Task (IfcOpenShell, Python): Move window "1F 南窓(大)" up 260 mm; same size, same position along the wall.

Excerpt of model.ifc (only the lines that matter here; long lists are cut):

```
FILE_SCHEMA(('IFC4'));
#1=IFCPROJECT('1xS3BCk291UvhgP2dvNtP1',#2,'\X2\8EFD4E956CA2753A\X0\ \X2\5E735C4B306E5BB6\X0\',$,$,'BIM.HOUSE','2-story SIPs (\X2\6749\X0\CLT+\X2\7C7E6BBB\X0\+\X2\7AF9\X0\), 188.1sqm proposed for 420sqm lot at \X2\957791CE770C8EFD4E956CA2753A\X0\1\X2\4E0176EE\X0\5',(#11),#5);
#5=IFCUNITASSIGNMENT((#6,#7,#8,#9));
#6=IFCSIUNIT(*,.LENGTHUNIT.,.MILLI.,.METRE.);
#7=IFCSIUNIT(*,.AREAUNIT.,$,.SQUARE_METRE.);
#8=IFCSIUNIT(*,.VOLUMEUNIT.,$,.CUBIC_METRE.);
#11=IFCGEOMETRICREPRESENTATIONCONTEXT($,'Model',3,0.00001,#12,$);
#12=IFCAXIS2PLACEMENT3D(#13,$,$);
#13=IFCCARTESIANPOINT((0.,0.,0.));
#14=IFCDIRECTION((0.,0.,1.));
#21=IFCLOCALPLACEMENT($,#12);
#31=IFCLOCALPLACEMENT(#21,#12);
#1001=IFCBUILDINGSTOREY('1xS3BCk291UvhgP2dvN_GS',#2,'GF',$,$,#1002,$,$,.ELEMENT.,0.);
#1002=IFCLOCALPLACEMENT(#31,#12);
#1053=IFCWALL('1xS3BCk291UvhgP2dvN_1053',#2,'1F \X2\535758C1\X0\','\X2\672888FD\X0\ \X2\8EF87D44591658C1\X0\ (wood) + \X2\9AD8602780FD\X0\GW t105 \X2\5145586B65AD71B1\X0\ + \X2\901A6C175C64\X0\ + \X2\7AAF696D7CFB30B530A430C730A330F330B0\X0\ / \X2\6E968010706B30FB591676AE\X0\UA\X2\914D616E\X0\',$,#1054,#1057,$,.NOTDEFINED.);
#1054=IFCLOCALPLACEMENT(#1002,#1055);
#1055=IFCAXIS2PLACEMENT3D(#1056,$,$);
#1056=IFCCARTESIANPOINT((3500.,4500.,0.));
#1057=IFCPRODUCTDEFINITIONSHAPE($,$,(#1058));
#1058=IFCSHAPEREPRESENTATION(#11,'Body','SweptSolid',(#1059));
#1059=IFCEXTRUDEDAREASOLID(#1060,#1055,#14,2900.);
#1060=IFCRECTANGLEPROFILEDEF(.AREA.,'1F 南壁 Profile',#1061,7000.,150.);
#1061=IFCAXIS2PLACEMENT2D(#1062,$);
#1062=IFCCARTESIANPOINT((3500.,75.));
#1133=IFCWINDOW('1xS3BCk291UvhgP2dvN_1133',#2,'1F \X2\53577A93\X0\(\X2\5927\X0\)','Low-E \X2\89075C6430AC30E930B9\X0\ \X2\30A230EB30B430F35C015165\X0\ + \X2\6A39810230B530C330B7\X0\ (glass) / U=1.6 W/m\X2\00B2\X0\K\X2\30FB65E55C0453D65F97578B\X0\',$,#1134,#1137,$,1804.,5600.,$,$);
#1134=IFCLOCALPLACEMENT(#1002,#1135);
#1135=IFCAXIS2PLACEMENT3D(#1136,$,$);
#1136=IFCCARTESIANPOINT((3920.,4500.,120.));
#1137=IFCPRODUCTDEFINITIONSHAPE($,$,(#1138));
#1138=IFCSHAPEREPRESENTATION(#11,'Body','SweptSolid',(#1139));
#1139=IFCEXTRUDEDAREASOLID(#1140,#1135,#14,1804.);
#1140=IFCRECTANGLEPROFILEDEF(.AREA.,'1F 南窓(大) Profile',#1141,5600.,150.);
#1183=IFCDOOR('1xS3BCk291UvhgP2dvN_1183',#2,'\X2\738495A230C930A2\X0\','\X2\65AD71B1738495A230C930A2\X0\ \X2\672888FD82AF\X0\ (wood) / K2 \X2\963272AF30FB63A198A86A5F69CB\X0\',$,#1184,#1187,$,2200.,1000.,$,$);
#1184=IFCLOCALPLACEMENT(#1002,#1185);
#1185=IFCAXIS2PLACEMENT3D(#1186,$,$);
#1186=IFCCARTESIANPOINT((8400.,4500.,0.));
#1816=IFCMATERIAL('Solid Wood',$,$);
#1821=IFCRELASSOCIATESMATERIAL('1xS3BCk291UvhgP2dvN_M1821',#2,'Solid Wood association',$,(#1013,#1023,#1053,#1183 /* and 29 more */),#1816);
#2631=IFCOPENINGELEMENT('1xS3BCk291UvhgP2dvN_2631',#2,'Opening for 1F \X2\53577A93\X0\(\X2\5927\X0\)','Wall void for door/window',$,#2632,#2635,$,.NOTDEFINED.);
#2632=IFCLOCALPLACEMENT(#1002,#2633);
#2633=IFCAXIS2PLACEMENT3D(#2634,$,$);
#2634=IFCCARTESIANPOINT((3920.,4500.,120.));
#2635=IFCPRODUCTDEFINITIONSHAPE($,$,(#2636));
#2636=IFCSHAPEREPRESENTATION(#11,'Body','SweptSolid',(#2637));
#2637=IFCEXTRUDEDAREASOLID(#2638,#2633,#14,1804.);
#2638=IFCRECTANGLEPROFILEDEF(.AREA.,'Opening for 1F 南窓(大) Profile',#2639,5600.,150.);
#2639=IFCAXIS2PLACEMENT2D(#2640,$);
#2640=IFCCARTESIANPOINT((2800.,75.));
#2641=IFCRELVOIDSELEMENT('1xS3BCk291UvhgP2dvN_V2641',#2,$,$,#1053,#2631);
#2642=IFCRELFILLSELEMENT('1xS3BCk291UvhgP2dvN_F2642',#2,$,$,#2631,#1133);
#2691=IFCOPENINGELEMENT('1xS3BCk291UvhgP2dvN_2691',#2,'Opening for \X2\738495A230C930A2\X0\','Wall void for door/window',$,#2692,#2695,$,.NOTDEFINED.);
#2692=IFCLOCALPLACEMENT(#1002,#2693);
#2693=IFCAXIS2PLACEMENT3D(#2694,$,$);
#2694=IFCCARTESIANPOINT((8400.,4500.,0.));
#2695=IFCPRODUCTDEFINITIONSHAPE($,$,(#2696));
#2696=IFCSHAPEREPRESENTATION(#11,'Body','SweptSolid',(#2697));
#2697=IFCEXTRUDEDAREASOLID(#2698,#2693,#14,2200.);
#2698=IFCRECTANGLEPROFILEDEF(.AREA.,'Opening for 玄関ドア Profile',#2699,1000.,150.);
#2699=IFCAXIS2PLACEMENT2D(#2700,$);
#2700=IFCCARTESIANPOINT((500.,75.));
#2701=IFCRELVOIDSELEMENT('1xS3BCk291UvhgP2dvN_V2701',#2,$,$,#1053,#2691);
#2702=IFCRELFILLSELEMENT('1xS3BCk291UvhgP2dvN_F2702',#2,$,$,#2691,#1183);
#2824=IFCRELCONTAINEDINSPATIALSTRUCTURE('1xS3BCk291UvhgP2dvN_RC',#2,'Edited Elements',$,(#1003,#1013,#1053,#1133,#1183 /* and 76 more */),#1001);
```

```python
import numpy as np
import ifcopenshell
import ifcopenshell.api.geometry
import ifcopenshell.util.placement
import ifcopenshell.util.unit

model = ifcopenshell.open("model.ifc")
unit_scale = ifcopenshell.util.unit.calculate_unit_scale(model)

window = model.by_id(1133)
opening = window.FillsVoids[0].RelatingOpeningElement
dz = 0.26 / unit_scale

shift = np.array([0.0, 0.0, dz])
# The window is not placed relative to its opening, so move both.
for product in (opening, window):
    matrix = ifcopenshell.util.placement.get_local_placement(product.ObjectPlacement)
    matrix[:3, 3] += shift
    ifcopenshell.api.geometry.edit_object_placement(model, product=product, matrix=matrix, is_si=False)

print(f"moved by {dz * unit_scale:+.3f} m")

model.write("model_v2.ifc")
```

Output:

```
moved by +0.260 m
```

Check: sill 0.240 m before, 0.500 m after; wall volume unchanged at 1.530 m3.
